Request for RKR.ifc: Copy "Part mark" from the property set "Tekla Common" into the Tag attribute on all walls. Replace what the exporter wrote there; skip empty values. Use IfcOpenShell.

First a look at what the model holds.

```python
import ifcopenshell
import ifcopenshell.util.element

model = ifcopenshell.open("RKR.ifc")
print(model.schema)
walls = model.by_type("IfcWall")
print(len(walls), "walls")
for e in walls[:8]:
    source = ifcopenshell.util.element.get_pset(e, "Tekla Common", "Part mark")
    target = e.Tag
    print(e.id(), repr(source), repr(target), sep=" | ")
```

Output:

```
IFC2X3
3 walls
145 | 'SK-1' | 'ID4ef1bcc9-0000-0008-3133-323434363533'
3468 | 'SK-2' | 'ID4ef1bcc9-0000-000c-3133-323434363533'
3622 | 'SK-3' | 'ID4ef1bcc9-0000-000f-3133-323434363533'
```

```python
import ifcopenshell
import ifcopenshell.util.element

model = ifcopenshell.open("RKR.ifc")

count = 0
for e in model.by_type("IfcWall"):
    value = ifcopenshell.util.element.get_pset(e, "Tekla Common", "Part mark")
    current = e.Tag
    if not value or not value.strip() or current == value:
        continue
    e.Tag = value
    count += 1

print(count, "walls updated")

model.write("RKR_edited.ifc")
```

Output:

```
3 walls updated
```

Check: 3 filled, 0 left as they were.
